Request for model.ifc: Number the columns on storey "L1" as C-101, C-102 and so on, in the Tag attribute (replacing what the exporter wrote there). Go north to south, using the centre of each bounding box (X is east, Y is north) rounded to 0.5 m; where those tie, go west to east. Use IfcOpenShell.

First a look at what the model holds.

```python
import ifcopenshell
import ifcopenshell.util.element
import ifcopenshell.util.placement

model = ifcopenshell.open("model.ifc")
print(model.schema)
storey = next(s for s in model.by_type("IfcBuildingStorey") if s.Name == "L1")
columns = [e for e in ifcopenshell.util.element.get_decomposition(storey) if e.is_a("IfcColumn")]
for e in sorted(columns, key=lambda e: e.id()):
    origin = ifcopenshell.util.placement.get_local_placement(e.ObjectPlacement)[:3, 3]
    print(e.id(), e.Tag, e.Name, origin.round(2) + 0.0, sep=" | ")
```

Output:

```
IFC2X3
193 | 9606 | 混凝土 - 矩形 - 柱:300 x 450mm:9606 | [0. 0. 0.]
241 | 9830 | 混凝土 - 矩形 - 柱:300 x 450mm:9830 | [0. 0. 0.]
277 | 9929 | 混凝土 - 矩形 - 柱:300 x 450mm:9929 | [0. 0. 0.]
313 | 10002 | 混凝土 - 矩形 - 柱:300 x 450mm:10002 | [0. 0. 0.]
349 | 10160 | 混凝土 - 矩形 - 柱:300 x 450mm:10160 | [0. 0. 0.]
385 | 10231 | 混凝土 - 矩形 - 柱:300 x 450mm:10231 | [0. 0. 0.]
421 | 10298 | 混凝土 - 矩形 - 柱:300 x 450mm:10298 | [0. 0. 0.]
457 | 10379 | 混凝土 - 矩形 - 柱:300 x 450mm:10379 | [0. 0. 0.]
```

```python
import ifcopenshell
import ifcopenshell.geom
import ifcopenshell.util.element
import ifcopenshell.util.shape

model = ifcopenshell.open("model.ifc")
settings = ifcopenshell.geom.settings()
settings.set("use-world-coords", True)


def centre(element):
    shape = ifcopenshell.geom.create_shape(settings, element)
    return ifcopenshell.util.shape.get_bbox_centroid(shape.geometry)


storey = next(s for s in model.by_type("IfcBuildingStorey") if s.Name == "L1")
columns = [e for e in ifcopenshell.util.element.get_decomposition(storey) if e.is_a("IfcColumn")]

# Insertion points can sit at a corner or the storey origin, so sort by the geometry (in metres).
centres = {e: centre(e) for e in columns}
columns.sort(key=lambda e: (-round(centres[e][1] / 0.5), centres[e][0]))

for i, e in enumerate(columns, start=1):
    number = f"C-1{i:02d}"
    e.Tag = number
    print(e.id(), number)

model.write("model_rev.ifc")
```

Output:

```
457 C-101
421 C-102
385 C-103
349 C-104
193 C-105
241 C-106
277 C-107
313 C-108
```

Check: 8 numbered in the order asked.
